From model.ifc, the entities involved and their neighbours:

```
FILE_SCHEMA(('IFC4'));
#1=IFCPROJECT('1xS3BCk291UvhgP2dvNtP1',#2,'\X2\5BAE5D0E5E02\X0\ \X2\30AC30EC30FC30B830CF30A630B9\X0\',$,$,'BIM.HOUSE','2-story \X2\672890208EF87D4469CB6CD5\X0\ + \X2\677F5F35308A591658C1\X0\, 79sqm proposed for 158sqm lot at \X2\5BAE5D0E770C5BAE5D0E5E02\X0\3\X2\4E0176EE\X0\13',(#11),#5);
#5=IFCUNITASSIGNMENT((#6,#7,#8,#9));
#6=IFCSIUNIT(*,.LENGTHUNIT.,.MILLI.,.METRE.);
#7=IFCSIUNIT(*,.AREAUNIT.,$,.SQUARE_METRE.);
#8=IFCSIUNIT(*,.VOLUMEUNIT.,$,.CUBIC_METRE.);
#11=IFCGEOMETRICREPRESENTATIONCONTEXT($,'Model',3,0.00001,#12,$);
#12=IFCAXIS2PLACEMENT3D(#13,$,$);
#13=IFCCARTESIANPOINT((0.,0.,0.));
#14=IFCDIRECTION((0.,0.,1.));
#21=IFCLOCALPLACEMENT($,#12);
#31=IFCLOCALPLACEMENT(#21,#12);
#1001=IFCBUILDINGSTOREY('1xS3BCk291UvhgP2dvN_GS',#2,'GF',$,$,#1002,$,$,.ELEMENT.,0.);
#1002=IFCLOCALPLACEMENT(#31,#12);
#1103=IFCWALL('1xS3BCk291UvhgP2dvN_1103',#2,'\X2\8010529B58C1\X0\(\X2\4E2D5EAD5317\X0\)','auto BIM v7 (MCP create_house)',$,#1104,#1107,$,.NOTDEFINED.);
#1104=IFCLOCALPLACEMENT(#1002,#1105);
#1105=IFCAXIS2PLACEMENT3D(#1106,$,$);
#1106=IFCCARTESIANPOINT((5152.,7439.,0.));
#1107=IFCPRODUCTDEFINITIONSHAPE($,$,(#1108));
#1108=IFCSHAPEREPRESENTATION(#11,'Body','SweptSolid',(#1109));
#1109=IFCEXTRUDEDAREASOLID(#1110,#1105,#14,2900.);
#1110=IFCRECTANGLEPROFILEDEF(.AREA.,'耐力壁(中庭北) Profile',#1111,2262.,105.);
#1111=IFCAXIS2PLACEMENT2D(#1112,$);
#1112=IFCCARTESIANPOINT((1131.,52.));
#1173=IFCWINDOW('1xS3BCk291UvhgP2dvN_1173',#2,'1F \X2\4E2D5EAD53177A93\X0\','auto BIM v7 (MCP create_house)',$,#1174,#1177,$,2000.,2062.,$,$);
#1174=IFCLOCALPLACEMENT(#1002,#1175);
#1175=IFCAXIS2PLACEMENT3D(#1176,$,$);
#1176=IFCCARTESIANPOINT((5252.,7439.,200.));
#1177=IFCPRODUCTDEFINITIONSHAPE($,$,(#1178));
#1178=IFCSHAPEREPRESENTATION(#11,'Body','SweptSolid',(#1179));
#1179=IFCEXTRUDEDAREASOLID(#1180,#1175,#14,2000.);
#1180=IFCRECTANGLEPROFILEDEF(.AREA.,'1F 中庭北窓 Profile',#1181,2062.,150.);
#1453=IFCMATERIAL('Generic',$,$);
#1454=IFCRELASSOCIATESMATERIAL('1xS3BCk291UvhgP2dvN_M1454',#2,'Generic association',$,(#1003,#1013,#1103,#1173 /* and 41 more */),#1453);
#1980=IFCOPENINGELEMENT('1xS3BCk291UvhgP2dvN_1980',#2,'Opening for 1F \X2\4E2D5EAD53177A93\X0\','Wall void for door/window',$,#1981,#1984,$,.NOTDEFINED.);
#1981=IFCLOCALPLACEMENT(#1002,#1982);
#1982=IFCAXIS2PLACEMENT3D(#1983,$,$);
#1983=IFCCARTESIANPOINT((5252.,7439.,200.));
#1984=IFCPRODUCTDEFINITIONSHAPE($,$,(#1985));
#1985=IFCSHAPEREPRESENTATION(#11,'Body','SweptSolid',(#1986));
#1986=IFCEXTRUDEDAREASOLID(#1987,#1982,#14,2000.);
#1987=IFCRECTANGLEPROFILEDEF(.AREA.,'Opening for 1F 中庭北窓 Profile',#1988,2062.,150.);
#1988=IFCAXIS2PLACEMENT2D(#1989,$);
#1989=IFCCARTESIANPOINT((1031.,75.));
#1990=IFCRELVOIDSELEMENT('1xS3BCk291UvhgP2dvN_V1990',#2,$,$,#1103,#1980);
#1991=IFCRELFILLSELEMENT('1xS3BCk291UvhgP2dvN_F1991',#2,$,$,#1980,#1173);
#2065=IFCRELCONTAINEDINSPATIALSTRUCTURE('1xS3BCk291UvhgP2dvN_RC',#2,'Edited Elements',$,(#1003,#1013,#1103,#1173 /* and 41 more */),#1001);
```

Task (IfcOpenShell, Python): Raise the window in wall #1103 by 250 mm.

```python
import numpy as np
import ifcopenshell
import ifcopenshell.api.geometry
import ifcopenshell.util.placement
import ifcopenshell.util.unit

model = ifcopenshell.open("model.ifc")
unit_scale = ifcopenshell.util.unit.calculate_unit_scale(model)

window = model.by_id(1173)
opening = window.FillsVoids[0].RelatingOpeningElement
dz = 250.0

shift = np.array([0.0, 0.0, dz])
# The window is not placed relative to its opening, so move both.
for product in (opening, window):
    matrix = ifcopenshell.util.placement.get_local_placement(product.ObjectPlacement)
    matrix[:3, 3] += shift
    ifcopenshell.api.geometry.edit_object_placement(model, product=product, matrix=matrix, is_si=False)

print(f"moved by {dz * unit_scale:+.3f} m")

model.write("model-out.ifc")
```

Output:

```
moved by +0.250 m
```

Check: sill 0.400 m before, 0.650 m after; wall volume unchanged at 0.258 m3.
